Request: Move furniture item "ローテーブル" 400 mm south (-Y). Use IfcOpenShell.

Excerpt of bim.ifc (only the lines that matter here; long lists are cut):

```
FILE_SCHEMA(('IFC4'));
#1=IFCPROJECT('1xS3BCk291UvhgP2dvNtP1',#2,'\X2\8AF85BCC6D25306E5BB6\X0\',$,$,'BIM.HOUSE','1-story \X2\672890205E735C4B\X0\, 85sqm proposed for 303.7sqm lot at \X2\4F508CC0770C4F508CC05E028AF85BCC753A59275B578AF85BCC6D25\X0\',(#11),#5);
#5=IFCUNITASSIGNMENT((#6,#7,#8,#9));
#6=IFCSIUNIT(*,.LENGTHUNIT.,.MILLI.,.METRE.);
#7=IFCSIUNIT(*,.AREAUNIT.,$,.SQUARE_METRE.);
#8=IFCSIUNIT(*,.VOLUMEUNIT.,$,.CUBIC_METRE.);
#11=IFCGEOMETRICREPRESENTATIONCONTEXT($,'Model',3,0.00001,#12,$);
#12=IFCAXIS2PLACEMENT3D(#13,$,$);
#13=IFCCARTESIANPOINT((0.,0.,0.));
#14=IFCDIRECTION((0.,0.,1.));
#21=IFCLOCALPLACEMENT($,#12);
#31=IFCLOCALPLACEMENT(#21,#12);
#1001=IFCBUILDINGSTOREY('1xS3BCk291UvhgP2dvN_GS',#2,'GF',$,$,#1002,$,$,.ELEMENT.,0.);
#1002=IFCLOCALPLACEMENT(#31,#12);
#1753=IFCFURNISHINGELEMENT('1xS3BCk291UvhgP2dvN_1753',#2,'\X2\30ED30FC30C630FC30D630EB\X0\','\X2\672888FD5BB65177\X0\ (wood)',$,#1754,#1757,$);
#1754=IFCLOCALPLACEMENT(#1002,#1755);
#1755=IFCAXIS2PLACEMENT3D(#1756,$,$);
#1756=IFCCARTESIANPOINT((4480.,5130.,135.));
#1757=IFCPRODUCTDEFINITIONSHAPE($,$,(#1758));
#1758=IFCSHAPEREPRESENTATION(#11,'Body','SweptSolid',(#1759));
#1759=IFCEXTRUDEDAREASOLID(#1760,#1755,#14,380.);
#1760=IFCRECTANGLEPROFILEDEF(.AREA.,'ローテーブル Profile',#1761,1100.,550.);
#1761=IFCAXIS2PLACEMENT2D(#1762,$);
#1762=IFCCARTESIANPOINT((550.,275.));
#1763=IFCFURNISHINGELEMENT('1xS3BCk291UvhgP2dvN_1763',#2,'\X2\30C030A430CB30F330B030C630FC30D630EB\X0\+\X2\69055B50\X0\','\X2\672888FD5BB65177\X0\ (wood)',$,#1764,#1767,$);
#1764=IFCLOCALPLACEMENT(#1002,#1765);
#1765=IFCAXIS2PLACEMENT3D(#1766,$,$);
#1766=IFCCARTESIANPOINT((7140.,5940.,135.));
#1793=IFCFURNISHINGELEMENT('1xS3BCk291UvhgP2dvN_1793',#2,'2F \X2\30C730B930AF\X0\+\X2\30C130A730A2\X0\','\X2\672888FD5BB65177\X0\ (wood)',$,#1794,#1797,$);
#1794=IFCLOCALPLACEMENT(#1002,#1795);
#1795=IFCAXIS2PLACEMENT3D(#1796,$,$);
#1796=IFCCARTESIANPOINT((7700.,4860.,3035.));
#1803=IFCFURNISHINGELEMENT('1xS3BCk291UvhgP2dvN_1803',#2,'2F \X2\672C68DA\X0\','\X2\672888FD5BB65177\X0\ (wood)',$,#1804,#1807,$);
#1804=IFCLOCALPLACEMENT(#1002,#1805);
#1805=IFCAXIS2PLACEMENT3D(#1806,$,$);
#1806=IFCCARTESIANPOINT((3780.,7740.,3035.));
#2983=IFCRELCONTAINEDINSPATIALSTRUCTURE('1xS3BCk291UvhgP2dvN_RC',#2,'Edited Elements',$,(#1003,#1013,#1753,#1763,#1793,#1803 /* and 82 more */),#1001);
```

```python
import ifcopenshell
import ifcopenshell.api.geometry
import ifcopenshell.util.placement
import ifcopenshell.util.unit

model = ifcopenshell.open("bim.ifc")
unit_scale = ifcopenshell.util.unit.calculate_unit_scale(model)

item = model.by_guid("1xS3BCk291UvhgP2dvN_1753")
matrix = ifcopenshell.util.placement.get_local_placement(item.ObjectPlacement)
matrix[1, 3] -= 0.4 / unit_scale
ifcopenshell.api.geometry.edit_object_placement(model, product=item, matrix=matrix, is_si=False)

print(ifcopenshell.util.placement.get_local_placement(item.ObjectPlacement).round(3) + 0.0)

model.write("bim_edited.ifc")
```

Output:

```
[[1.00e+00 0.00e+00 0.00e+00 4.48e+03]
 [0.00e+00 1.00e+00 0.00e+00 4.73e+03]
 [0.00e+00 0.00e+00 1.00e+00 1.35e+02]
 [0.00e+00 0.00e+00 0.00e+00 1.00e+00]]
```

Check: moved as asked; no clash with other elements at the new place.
